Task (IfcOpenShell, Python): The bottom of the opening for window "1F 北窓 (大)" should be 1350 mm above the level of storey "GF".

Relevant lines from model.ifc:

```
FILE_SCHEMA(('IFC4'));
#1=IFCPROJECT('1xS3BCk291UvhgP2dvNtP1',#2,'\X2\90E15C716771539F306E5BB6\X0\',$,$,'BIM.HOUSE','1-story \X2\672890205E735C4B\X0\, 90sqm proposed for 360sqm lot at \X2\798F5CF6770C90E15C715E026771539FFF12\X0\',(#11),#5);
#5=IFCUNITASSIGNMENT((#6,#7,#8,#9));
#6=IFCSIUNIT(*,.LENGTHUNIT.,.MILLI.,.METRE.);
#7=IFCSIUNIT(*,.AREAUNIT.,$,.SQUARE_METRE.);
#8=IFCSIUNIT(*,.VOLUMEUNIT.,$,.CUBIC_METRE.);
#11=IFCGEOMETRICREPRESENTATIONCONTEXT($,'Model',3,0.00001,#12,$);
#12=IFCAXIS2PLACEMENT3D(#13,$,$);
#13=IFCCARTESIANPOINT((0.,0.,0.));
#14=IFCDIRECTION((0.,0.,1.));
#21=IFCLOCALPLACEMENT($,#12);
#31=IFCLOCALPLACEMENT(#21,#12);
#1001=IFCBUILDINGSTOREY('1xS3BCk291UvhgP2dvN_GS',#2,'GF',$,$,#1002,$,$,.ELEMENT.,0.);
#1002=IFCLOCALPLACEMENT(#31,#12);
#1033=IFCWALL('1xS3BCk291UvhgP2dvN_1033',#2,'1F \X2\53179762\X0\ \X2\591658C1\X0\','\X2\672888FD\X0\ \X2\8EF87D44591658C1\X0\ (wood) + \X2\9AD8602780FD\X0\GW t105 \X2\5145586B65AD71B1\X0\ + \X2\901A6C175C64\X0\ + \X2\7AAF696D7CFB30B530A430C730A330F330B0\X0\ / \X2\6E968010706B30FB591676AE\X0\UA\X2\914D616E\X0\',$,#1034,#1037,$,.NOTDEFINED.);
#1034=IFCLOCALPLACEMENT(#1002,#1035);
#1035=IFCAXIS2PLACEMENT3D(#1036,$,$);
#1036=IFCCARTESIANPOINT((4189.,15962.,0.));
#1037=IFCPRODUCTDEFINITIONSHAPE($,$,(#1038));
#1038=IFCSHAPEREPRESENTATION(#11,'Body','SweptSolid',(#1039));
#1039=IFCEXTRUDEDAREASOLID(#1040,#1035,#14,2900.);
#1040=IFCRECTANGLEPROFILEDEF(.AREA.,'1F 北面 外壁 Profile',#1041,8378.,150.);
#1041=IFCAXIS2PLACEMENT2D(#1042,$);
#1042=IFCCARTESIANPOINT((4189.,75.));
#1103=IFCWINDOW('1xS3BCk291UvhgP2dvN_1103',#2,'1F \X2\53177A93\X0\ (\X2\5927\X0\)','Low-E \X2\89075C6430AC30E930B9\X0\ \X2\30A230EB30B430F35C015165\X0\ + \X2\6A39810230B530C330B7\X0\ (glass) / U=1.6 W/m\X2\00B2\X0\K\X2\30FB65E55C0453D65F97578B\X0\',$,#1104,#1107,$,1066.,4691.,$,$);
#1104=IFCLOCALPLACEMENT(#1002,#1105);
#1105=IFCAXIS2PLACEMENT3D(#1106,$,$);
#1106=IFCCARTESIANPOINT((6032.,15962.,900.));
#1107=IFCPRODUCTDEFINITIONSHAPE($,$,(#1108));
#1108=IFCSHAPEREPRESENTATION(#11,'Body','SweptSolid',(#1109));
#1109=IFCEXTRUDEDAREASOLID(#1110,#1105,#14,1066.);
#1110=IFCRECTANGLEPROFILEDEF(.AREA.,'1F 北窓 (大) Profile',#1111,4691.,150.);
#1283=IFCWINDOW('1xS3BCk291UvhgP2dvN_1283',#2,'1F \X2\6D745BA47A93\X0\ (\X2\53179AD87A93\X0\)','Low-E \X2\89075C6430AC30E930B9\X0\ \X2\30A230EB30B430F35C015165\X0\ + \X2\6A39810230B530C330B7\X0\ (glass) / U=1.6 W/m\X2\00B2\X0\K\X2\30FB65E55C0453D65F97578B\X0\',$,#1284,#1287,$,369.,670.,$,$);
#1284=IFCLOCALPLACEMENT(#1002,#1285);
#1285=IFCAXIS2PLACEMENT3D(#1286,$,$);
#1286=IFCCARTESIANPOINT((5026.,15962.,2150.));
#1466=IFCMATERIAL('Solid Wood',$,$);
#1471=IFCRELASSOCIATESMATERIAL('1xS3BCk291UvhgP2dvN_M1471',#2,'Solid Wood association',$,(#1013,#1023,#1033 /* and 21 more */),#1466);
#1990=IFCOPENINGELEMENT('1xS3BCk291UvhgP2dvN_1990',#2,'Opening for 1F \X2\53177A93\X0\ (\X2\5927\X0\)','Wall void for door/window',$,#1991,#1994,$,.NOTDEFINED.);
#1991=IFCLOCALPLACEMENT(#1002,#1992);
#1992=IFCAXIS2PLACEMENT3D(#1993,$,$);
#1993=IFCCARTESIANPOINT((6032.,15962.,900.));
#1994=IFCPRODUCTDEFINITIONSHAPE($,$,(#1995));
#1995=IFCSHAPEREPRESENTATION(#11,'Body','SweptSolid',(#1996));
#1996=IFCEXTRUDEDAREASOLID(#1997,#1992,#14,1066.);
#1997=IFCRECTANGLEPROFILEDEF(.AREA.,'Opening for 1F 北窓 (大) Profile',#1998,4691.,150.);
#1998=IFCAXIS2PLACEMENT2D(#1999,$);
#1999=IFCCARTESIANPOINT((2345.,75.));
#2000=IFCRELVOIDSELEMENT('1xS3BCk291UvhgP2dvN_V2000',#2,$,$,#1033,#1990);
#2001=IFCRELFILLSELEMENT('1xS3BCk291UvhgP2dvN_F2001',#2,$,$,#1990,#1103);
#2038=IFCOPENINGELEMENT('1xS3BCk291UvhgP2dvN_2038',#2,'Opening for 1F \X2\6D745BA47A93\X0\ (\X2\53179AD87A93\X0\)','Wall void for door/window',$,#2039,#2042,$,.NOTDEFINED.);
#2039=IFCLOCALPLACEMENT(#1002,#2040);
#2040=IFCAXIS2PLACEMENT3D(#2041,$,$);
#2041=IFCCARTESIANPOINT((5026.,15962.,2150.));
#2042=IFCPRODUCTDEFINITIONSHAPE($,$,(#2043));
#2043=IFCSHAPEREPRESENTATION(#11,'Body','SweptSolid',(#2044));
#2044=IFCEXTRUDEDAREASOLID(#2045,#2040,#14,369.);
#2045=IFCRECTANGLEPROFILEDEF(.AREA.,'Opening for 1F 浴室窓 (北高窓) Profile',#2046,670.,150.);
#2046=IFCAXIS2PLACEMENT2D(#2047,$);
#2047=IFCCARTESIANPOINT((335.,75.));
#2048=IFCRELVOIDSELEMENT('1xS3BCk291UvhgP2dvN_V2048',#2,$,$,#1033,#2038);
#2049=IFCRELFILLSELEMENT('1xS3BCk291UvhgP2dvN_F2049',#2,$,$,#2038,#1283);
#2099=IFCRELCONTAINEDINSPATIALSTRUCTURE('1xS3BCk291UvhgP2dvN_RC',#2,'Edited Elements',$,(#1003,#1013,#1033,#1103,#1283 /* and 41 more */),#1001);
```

```python
import numpy as np
import ifcopenshell
import ifcopenshell.api.geometry
import ifcopenshell.geom
import ifcopenshell.util.element
import ifcopenshell.util.placement
import ifcopenshell.util.shape
import ifcopenshell.util.unit

model = ifcopenshell.open("model.ifc")
unit_scale = ifcopenshell.util.unit.calculate_unit_scale(model)

window = model.by_id(1103)
opening = window.FillsVoids[0].RelatingOpeningElement
storey = ifcopenshell.util.element.get_container(window, ifc_class="IfcBuildingStorey")
level = ifcopenshell.util.placement.get_local_placement(storey.ObjectPlacement)[2, 3]

# The opening's origin need not be at the sill, so measure its lowest point.
shape = ifcopenshell.geom.create_shape(ifcopenshell.geom.settings(), opening)
bottom = ifcopenshell.util.shape.get_shape_bottom_elevation(shape, shape.geometry) / unit_scale
dz = level + 1350.0 - bottom

shift = np.array([0.0, 0.0, dz])
# The window is not placed relative to its opening, so move both.
for product in (opening, window):
    matrix = ifcopenshell.util.placement.get_local_placement(product.ObjectPlacement)
    matrix[:3, 3] += shift
    ifcopenshell.api.geometry.edit_object_placement(model, product=product, matrix=matrix, is_si=False)

print(f"moved by {dz * unit_scale:+.3f} m")

model.write("model_rev.ifc")
```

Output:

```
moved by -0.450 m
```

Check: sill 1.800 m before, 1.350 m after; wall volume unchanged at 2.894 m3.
